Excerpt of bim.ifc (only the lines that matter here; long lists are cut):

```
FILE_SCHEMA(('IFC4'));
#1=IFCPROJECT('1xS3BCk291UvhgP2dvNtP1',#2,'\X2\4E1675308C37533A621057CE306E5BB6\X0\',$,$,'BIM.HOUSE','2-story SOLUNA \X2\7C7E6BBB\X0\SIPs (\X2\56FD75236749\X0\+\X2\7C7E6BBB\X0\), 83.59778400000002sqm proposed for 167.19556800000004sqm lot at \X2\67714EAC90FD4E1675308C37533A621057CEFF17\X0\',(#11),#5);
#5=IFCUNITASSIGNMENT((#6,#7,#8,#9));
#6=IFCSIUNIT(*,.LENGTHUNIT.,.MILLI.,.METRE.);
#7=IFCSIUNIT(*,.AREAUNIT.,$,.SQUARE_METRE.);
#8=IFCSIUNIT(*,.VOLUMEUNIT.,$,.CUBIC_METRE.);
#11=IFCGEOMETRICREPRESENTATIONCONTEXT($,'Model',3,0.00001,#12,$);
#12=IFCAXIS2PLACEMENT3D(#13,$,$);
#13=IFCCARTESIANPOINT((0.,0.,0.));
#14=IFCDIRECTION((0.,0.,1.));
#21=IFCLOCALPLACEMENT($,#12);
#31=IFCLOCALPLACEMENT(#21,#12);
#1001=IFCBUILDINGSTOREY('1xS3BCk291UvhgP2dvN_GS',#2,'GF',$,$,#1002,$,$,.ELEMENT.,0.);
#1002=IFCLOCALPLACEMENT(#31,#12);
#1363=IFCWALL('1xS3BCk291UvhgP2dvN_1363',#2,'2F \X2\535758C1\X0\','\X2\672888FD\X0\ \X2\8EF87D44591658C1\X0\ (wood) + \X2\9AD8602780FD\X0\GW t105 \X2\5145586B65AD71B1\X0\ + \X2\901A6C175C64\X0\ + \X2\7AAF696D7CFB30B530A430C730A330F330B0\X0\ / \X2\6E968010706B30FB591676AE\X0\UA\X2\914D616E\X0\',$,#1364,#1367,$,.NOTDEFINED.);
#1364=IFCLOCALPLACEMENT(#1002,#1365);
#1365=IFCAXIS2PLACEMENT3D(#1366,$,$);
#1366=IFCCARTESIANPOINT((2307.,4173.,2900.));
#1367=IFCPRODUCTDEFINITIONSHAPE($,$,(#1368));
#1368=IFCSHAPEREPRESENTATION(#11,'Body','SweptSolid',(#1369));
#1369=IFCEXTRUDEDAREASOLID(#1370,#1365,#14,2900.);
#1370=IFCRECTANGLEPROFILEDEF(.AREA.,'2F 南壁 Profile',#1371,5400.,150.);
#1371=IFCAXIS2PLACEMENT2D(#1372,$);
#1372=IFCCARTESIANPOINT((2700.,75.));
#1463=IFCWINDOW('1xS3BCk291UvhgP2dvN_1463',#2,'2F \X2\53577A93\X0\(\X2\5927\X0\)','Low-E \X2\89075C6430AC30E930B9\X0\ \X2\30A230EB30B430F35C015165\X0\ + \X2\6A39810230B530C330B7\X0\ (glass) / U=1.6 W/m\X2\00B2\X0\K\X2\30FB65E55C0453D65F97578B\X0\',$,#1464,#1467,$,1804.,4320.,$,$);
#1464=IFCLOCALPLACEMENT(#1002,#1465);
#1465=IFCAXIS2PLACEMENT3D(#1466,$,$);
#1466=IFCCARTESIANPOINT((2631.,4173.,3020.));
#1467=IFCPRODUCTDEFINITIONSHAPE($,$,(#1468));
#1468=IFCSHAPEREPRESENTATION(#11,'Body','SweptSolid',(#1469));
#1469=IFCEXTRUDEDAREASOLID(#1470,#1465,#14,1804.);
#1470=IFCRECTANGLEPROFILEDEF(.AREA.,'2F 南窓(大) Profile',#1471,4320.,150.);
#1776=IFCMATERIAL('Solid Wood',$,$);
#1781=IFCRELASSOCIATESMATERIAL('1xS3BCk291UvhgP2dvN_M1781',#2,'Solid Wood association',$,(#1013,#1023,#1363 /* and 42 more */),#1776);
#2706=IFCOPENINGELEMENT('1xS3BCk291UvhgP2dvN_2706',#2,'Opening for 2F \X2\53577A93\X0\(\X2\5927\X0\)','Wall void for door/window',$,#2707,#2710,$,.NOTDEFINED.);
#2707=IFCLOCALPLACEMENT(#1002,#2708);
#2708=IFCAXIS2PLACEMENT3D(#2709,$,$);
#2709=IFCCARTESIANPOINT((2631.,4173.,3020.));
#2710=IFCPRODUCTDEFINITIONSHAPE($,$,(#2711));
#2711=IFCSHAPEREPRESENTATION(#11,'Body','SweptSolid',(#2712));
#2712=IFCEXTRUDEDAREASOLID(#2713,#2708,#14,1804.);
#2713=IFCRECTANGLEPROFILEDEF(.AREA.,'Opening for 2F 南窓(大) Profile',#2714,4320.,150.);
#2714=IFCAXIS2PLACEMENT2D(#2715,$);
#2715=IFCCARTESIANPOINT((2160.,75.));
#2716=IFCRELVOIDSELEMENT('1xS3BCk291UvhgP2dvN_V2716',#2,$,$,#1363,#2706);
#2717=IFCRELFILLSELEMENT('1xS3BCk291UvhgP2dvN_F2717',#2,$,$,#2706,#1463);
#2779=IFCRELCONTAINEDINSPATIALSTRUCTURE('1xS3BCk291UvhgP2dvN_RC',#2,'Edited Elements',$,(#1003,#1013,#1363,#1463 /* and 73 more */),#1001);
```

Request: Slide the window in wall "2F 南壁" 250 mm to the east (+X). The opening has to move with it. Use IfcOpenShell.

```python
import ifcopenshell
import ifcopenshell.api.geometry
import ifcopenshell.util.placement
import ifcopenshell.util.unit

model = ifcopenshell.open("bim.ifc")
unit_scale = ifcopenshell.util.unit.calculate_unit_scale(model)

window = model.by_guid("1xS3BCk291UvhgP2dvN_1463")
opening = window.FillsVoids[0].RelatingOpeningElement
wall = opening.VoidsElements[0].RelatingBuildingElement

wall_matrix = ifcopenshell.util.placement.get_local_placement(wall.ObjectPlacement)
shift = wall_matrix[:3, 0] * 0.25 / unit_scale
before = ifcopenshell.util.placement.get_local_placement(window.ObjectPlacement)[:3, 3].copy()

# The window is not placed relative to its opening, so move both.
for product in (opening, window):
    matrix = ifcopenshell.util.placement.get_local_placement(product.ObjectPlacement)
    matrix[:3, 3] += shift
    ifcopenshell.api.geometry.edit_object_placement(model, product=product, matrix=matrix, is_si=False)

after = ifcopenshell.util.placement.get_local_placement(window.ObjectPlacement)[:3, 3]
print("window moved by", (after - before).round(3) + 0.0)

model.write("bim_rev.ifc")
```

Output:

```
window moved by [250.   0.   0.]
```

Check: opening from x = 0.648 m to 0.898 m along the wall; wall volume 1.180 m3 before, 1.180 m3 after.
